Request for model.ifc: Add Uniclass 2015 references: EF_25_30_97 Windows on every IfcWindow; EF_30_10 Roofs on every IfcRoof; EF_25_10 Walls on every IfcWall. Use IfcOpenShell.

First a look at what the model holds.

```python
import ifcopenshell

model = ifcopenshell.open("model.ifc")
print(model.schema)
print("classifications:", [c.Name for c in model.by_type("IfcClassification")])
for ifc_class in ("IfcDoor", "IfcRoof", "IfcStair", "IfcWall", "IfcWindow"):
    print(ifc_class, len(model.by_type(ifc_class)))
```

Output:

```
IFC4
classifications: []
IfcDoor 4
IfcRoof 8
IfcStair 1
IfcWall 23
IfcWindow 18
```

```python
import ifcopenshell
import ifcopenshell.api.classification

model = ifcopenshell.open("model.ifc")

system = ifcopenshell.api.classification.add_classification(model, classification="Uniclass 2015")

codes = {
    "IfcWindow": ("EF_25_30_97", "Windows"),
    "IfcRoof": ("EF_30_10", "Roofs"),
    "IfcWall": ("EF_25_10", "Walls"),
}
for ifc_class, (code, name) in codes.items():
    products = model.by_type(ifc_class)
    ifcopenshell.api.classification.add_reference(
        model, products=products, classification=system, identification=code, name=name
    )
    print(code, len(products))

model.write("model_v2.ifc")
```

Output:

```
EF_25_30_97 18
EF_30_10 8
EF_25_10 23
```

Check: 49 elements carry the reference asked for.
